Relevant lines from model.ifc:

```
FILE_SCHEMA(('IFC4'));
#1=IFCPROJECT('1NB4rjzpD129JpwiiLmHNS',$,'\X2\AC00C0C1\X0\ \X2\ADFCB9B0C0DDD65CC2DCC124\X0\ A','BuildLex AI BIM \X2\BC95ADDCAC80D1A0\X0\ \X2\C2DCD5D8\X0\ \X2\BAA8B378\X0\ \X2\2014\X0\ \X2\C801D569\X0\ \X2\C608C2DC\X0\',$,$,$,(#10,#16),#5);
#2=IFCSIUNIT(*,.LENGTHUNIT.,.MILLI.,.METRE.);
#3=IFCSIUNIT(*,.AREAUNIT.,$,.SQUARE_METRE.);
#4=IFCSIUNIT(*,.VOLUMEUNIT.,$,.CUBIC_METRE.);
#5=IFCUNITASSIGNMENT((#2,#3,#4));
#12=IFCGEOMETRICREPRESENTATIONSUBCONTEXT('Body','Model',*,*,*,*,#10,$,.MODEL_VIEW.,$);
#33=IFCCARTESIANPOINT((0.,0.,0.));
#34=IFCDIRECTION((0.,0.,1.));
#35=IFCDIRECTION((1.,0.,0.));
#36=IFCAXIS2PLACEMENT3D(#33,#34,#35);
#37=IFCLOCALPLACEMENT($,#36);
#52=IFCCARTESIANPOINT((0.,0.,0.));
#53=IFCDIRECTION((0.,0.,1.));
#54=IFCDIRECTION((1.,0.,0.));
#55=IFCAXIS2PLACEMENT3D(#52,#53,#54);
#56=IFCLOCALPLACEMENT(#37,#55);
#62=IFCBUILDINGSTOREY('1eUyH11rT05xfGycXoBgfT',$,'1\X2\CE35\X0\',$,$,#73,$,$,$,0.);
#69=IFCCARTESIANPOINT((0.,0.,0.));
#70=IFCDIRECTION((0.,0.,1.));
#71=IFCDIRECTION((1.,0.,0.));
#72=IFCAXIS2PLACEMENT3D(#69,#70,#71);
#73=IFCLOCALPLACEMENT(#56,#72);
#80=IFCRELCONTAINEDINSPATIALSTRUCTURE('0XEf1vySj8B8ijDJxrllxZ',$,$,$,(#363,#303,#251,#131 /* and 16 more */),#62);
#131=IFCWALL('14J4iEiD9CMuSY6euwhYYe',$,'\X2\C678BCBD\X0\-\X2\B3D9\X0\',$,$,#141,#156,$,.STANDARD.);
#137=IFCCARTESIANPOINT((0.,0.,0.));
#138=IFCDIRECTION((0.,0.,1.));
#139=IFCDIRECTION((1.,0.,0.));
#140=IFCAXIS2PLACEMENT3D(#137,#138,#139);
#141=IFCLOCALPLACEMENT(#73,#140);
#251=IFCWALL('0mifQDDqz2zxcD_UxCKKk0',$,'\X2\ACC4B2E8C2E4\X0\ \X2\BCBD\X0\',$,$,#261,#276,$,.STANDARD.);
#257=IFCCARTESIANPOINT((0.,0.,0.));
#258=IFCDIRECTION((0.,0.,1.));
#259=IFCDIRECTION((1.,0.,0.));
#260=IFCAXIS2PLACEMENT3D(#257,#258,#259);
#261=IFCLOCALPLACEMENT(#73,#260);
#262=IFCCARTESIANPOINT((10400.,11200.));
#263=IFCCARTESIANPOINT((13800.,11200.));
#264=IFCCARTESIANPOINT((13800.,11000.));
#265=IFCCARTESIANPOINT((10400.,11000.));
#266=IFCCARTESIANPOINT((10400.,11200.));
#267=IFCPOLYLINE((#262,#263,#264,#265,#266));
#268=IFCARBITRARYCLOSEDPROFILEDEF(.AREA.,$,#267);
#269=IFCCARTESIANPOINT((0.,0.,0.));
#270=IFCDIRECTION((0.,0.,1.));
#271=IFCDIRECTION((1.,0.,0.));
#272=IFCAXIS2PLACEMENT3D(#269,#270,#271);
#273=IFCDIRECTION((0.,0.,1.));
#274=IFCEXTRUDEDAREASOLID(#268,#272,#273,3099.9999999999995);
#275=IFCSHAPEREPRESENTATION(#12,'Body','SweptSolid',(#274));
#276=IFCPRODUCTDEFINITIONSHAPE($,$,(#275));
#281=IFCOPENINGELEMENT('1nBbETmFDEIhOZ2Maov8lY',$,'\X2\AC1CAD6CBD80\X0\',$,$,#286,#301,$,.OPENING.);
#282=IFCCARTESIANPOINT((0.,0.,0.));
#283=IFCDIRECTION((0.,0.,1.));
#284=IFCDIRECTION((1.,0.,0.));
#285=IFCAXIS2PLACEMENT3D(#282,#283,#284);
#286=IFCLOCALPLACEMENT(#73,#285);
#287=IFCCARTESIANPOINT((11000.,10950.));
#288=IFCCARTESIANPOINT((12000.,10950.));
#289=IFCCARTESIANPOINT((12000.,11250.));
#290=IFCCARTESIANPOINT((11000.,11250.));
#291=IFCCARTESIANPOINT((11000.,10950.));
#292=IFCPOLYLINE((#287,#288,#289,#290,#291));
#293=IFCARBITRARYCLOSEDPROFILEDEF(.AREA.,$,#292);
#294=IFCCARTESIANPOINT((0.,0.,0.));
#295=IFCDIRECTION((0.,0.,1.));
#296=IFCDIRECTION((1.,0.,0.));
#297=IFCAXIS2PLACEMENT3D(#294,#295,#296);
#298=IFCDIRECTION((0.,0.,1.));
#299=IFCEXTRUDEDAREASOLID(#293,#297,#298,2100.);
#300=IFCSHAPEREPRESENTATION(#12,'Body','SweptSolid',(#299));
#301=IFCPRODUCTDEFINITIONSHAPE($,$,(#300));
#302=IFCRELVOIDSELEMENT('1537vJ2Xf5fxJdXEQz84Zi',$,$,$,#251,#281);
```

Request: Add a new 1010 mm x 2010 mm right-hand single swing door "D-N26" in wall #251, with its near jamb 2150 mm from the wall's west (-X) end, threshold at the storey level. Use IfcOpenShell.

```python
import numpy as np
import ifcopenshell
import ifcopenshell.api.feature
import ifcopenshell.api.geometry
import ifcopenshell.api.root
import ifcopenshell.api.spatial
import ifcopenshell.geom
import ifcopenshell.util.element
import ifcopenshell.util.placement
import ifcopenshell.util.representation
import ifcopenshell.util.shape
import ifcopenshell.util.unit

model = ifcopenshell.open("model.ifc")
unit_scale = ifcopenshell.util.unit.calculate_unit_scale(model)
settings = ifcopenshell.geom.settings()


def volume(element):
    """Net volume in cubic metres, openings subtracted."""
    shape = ifcopenshell.geom.create_shape(settings, element)
    return ifcopenshell.util.shape.get_volume(shape.geometry)


wall = model.by_id(251)
storey = ifcopenshell.util.element.get_container(wall, ifc_class="IfcBuildingStorey")
context = ifcopenshell.util.representation.get_context(model, "Model", "Body", "MODEL_VIEW")
before = volume(wall)

width, height, from_end, sill = 1.01, 2.01, 2.15, 0.0  # metres

# The wall runs along its own X axis, and the end named is its -X end.
wall_shape = ifcopenshell.geom.create_shape(settings, wall)
x, y, z = ifcopenshell.util.shape.get_vertices(wall_shape.geometry).T
start = x.min() + from_end
face, thickness = float(y.min()), float(y.max() - y.min())
wall_matrix = ifcopenshell.util.placement.get_local_placement(wall.ObjectPlacement)
level = ifcopenshell.util.placement.get_local_placement(storey.ObjectPlacement)[2, 3]


def in_wall(x, y):
    """Placement at x, y metres in the wall's axes, at sill height."""
    matrix = wall_matrix.copy()
    matrix[:, 3] = wall_matrix @ np.array([x / unit_scale, y / unit_scale, 0.0, 1.0])
    matrix[2, 3] = level + sill / unit_scale
    return matrix


# Opening: a box that overshoots both wall faces by 50 mm.
opening = ifcopenshell.api.root.create_entity(model, ifc_class="IfcOpeningElement", predefined_type="OPENING")
box = ifcopenshell.api.geometry.add_wall_representation(
    model, context=context, length=width, height=height, thickness=thickness + 0.1
)
ifcopenshell.api.geometry.assign_representation(model, product=opening, representation=box)
ifcopenshell.api.geometry.edit_object_placement(model, product=opening, matrix=in_wall(start, face - 0.05), is_si=False)
ifcopenshell.api.feature.add_feature(model, feature=opening, element=wall)

door = ifcopenshell.api.root.create_entity(model, ifc_class="IfcDoor", name="D-N26", predefined_type="DOOR")
door.OverallWidth, door.OverallHeight = width / unit_scale, height / unit_scale
door.OperationType = "SINGLE_SWING_RIGHT"
body = ifcopenshell.api.geometry.add_door_representation(
    model,
    context=context,
    overall_width=door.OverallWidth,
    overall_height=door.OverallHeight,
    operation_type="SINGLE_SWING_RIGHT",
    lining_properties={"LiningDepth": thickness / unit_scale, "ThresholdDepth": thickness / unit_scale},
)
ifcopenshell.api.geometry.assign_representation(model, product=door, representation=body)
ifcopenshell.api.spatial.assign_container(model, products=[door], relating_structure=storey)
ifcopenshell.api.feature.add_filling(model, opening=opening, element=door)

# The lining spans the wall, so the door starts at the wall face.
ifcopenshell.api.geometry.edit_object_placement(model, product=door, matrix=in_wall(start, face), is_si=False)

after = volume(wall)

print(f"wall volume {before:.3f} -> {after:.3f} m3")

model.write("model-out.ifc")
```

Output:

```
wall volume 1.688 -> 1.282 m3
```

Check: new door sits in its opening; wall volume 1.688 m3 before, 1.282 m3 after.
